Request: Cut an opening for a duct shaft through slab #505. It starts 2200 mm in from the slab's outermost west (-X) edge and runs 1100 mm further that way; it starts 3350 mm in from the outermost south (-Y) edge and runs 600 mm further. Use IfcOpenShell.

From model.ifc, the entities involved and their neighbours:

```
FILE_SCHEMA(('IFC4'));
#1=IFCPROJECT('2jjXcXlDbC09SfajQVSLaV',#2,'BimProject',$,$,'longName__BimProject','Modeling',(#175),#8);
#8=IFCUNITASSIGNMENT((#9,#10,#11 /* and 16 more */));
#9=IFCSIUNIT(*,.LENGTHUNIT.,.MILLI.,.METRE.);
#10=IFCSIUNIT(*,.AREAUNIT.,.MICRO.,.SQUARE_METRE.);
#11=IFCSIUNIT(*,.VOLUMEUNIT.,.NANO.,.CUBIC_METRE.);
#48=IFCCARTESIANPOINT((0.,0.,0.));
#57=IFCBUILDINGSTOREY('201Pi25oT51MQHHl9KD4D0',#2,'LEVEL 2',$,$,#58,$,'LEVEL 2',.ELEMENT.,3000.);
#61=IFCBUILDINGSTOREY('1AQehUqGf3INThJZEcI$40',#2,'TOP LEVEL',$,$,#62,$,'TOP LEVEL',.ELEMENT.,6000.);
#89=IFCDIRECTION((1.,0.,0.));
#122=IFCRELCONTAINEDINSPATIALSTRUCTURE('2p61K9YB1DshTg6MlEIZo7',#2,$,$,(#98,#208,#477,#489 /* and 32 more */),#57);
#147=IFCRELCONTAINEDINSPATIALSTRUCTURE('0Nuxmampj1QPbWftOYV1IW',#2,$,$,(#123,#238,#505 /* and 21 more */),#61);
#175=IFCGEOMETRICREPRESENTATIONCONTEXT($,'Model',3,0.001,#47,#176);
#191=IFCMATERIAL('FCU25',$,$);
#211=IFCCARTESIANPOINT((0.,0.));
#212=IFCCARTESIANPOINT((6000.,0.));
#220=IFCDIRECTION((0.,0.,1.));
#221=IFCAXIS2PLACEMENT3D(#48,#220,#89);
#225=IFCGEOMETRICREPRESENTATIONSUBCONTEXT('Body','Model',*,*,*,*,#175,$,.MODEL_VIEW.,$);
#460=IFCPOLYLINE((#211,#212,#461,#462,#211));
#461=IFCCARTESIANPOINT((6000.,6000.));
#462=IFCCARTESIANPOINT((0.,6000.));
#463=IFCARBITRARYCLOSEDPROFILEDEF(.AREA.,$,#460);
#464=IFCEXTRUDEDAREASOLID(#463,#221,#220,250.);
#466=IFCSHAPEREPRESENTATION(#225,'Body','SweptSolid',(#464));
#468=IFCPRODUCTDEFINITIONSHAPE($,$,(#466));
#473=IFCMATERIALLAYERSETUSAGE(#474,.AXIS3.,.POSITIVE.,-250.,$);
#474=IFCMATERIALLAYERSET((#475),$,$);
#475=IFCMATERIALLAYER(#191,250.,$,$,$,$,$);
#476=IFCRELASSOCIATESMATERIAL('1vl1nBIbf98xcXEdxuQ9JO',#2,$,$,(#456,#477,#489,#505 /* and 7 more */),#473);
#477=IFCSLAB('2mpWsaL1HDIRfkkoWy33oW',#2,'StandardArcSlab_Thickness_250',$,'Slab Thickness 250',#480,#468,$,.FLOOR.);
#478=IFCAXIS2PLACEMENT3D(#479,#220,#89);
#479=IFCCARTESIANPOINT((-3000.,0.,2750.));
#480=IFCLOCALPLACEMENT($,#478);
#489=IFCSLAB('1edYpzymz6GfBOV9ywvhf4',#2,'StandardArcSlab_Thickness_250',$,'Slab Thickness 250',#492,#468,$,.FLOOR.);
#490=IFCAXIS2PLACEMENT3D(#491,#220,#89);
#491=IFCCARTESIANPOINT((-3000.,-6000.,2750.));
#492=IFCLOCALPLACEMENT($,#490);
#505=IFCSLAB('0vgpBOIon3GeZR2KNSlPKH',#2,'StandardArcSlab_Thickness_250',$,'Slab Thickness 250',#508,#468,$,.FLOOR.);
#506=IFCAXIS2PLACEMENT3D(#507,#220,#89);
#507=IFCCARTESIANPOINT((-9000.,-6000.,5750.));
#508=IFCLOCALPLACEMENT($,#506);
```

```python
import numpy as np
import ifcopenshell
import ifcopenshell.api.feature
import ifcopenshell.api.geometry
import ifcopenshell.api.root
import ifcopenshell.geom
import ifcopenshell.util.placement
import ifcopenshell.util.representation
import ifcopenshell.util.shape
import ifcopenshell.util.unit

model = ifcopenshell.open("model.ifc")
unit_scale = ifcopenshell.util.unit.calculate_unit_scale(model)
settings = ifcopenshell.geom.settings()


def volume(element):
    """Net volume in cubic metres, openings subtracted."""
    shape = ifcopenshell.geom.create_shape(settings, element)
    return ifcopenshell.util.shape.get_volume(shape.geometry)


slab = model.by_id(505)
before = volume(slab)

# Extent in the slab's own axes, in metres. The edges named are its -X and -Y sides.
slab_shape = ifcopenshell.geom.create_shape(settings, slab)
vertices = ifcopenshell.util.shape.get_vertices(slab_shape.geometry)
x_min, y_min, bottom = vertices.min(axis=0)
top = vertices[:, 2].max()

opening = ifcopenshell.api.root.create_entity(model, ifc_class="IfcOpeningElement", name="Duct shaft opening", predefined_type="OPENING")
context = ifcopenshell.util.representation.get_context(model, "Model", "Body", "MODEL_VIEW")
width, depth = 1.1, 0.6
outline = [(0.0, 0.0), (width, 0.0), (width, depth), (0.0, depth), (0.0, 0.0)]
# Overshoot both faces by 50 mm so the cut is clean.
shape = ifcopenshell.api.geometry.add_slab_representation(
    model, context=context, depth=top - bottom + 0.1, polyline=outline
)
ifcopenshell.api.geometry.assign_representation(model, product=opening, representation=shape)

matrix = ifcopenshell.util.placement.get_local_placement(slab.ObjectPlacement)
matrix[:, 3] = matrix @ np.append(np.array([x_min + 2.2, y_min + 3.35, bottom - 0.05]) / unit_scale, 1.0)
ifcopenshell.api.geometry.edit_object_placement(model, product=opening, matrix=matrix, is_si=False)
ifcopenshell.api.feature.add_feature(model, feature=opening, element=slab)

after = volume(slab)

print(f"slab volume {before:.3f} -> {after:.3f} m3")

model.write("model-out.ifc")
```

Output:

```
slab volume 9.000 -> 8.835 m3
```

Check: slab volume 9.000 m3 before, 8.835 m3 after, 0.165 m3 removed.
